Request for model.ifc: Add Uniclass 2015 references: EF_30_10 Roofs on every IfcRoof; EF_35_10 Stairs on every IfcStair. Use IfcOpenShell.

First a look at what the model holds.

```python
import ifcopenshell

model = ifcopenshell.open("model.ifc")
print(model.schema)
print("classifications:", [c.Name for c in model.by_type("IfcClassification")])
for ifc_class in ("IfcDoor", "IfcRoof", "IfcStair", "IfcWall", "IfcWindow"):
    print(ifc_class, len(model.by_type(ifc_class)))
```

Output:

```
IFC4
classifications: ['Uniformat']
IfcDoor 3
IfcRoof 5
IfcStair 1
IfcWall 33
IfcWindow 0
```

```python
import ifcopenshell
import ifcopenshell.api.classification

model = ifcopenshell.open("model.ifc")

system = ifcopenshell.api.classification.add_classification(model, classification="Uniclass 2015")

codes = {
    "IfcRoof": ("EF_30_10", "Roofs"),
    "IfcStair": ("EF_35_10", "Stairs"),
}
for ifc_class, (code, name) in codes.items():
    products = model.by_type(ifc_class)
    ifcopenshell.api.classification.add_reference(
        model, products=products, classification=system, identification=code, name=name
    )
    print(code, len(products))

model.write("model-out.ifc")
```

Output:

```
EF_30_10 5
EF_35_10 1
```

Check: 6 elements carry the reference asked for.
